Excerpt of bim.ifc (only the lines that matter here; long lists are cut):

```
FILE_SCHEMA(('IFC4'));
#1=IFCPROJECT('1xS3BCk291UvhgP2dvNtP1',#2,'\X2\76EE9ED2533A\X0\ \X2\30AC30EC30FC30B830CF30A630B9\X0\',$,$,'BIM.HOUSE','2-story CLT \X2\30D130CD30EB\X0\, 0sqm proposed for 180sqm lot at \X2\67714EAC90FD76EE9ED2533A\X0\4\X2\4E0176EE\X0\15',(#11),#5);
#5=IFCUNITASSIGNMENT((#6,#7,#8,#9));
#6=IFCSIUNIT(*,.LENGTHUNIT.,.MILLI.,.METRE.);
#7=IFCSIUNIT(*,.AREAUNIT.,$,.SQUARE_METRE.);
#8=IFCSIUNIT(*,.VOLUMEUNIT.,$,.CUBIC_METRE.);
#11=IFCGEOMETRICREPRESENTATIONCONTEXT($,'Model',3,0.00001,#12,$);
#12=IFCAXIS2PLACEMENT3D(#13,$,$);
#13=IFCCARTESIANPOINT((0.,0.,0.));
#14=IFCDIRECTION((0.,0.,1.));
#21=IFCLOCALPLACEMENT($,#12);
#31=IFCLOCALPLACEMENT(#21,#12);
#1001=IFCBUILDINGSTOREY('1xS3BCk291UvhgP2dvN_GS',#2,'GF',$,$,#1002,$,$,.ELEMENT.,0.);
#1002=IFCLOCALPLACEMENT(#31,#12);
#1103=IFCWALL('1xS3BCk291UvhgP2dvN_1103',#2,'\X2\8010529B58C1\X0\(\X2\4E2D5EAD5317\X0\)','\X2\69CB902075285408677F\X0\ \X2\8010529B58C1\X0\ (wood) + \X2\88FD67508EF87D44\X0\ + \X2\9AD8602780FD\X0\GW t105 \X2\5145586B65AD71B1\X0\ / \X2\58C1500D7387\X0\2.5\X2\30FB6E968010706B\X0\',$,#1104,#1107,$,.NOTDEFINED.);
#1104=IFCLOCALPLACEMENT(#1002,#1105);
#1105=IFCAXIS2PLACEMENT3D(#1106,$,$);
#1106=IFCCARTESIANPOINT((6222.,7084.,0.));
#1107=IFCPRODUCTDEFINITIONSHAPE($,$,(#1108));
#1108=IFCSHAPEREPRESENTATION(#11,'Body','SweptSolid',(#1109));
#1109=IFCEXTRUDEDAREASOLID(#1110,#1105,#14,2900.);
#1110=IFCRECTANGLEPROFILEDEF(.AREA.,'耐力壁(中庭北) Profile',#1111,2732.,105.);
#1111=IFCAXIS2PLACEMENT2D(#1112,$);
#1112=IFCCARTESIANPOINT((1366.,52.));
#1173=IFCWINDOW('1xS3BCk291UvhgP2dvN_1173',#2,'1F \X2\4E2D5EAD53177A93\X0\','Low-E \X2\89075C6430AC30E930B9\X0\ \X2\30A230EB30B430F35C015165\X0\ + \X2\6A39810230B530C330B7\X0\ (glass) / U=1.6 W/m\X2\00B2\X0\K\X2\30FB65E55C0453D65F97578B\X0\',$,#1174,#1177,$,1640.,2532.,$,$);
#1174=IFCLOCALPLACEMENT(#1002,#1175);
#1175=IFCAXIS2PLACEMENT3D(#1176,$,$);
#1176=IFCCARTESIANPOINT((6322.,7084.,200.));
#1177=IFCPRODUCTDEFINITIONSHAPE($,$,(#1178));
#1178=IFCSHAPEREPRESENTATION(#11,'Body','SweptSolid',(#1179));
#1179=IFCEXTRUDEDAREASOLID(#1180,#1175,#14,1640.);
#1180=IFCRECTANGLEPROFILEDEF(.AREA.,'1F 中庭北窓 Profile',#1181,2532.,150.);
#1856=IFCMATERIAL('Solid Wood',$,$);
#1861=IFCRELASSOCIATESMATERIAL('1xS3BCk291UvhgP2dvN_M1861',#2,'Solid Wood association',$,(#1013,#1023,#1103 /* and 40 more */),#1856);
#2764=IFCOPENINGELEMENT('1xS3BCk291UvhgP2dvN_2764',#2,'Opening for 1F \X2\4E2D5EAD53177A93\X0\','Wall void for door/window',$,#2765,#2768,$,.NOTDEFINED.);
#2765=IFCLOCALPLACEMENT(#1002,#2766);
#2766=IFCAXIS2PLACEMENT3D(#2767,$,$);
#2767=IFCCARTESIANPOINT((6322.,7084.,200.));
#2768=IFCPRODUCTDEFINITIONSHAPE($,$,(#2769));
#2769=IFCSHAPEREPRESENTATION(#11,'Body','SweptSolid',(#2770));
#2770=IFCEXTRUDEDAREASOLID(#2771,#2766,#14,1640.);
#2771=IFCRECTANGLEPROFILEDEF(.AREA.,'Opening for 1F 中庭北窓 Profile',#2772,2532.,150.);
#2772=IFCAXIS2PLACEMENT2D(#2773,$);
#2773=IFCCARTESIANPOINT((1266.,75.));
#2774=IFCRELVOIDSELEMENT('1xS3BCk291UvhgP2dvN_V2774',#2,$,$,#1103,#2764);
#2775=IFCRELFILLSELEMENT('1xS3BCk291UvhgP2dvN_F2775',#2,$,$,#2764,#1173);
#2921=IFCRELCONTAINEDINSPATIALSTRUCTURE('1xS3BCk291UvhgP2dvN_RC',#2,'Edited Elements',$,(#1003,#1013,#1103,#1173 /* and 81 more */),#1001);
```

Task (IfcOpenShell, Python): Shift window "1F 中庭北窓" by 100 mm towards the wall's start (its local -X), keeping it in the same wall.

```python
import ifcopenshell
import ifcopenshell.api.geometry
import ifcopenshell.util.placement
import ifcopenshell.util.unit

model = ifcopenshell.open("bim.ifc")
unit_scale = ifcopenshell.util.unit.calculate_unit_scale(model)

window = model.by_guid("1xS3BCk291UvhgP2dvN_1173")
opening = window.FillsVoids[0].RelatingOpeningElement
wall = opening.VoidsElements[0].RelatingBuildingElement

wall_matrix = ifcopenshell.util.placement.get_local_placement(wall.ObjectPlacement)
shift = wall_matrix[:3, 0] * -0.1 / unit_scale
before = ifcopenshell.util.placement.get_local_placement(window.ObjectPlacement)[:3, 3].copy()

# The window is not placed relative to its opening, so move both.
for product in (opening, window):
    matrix = ifcopenshell.util.placement.get_local_placement(product.ObjectPlacement)
    matrix[:3, 3] += shift
    ifcopenshell.api.geometry.edit_object_placement(model, product=product, matrix=matrix, is_si=False)

after = ifcopenshell.util.placement.get_local_placement(window.ObjectPlacement)[:3, 3]
print("window moved by", (after - before).round(3) + 0.0)

model.write("bim-out.ifc")
```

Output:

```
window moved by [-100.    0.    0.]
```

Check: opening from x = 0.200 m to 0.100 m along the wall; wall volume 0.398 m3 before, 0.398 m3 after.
